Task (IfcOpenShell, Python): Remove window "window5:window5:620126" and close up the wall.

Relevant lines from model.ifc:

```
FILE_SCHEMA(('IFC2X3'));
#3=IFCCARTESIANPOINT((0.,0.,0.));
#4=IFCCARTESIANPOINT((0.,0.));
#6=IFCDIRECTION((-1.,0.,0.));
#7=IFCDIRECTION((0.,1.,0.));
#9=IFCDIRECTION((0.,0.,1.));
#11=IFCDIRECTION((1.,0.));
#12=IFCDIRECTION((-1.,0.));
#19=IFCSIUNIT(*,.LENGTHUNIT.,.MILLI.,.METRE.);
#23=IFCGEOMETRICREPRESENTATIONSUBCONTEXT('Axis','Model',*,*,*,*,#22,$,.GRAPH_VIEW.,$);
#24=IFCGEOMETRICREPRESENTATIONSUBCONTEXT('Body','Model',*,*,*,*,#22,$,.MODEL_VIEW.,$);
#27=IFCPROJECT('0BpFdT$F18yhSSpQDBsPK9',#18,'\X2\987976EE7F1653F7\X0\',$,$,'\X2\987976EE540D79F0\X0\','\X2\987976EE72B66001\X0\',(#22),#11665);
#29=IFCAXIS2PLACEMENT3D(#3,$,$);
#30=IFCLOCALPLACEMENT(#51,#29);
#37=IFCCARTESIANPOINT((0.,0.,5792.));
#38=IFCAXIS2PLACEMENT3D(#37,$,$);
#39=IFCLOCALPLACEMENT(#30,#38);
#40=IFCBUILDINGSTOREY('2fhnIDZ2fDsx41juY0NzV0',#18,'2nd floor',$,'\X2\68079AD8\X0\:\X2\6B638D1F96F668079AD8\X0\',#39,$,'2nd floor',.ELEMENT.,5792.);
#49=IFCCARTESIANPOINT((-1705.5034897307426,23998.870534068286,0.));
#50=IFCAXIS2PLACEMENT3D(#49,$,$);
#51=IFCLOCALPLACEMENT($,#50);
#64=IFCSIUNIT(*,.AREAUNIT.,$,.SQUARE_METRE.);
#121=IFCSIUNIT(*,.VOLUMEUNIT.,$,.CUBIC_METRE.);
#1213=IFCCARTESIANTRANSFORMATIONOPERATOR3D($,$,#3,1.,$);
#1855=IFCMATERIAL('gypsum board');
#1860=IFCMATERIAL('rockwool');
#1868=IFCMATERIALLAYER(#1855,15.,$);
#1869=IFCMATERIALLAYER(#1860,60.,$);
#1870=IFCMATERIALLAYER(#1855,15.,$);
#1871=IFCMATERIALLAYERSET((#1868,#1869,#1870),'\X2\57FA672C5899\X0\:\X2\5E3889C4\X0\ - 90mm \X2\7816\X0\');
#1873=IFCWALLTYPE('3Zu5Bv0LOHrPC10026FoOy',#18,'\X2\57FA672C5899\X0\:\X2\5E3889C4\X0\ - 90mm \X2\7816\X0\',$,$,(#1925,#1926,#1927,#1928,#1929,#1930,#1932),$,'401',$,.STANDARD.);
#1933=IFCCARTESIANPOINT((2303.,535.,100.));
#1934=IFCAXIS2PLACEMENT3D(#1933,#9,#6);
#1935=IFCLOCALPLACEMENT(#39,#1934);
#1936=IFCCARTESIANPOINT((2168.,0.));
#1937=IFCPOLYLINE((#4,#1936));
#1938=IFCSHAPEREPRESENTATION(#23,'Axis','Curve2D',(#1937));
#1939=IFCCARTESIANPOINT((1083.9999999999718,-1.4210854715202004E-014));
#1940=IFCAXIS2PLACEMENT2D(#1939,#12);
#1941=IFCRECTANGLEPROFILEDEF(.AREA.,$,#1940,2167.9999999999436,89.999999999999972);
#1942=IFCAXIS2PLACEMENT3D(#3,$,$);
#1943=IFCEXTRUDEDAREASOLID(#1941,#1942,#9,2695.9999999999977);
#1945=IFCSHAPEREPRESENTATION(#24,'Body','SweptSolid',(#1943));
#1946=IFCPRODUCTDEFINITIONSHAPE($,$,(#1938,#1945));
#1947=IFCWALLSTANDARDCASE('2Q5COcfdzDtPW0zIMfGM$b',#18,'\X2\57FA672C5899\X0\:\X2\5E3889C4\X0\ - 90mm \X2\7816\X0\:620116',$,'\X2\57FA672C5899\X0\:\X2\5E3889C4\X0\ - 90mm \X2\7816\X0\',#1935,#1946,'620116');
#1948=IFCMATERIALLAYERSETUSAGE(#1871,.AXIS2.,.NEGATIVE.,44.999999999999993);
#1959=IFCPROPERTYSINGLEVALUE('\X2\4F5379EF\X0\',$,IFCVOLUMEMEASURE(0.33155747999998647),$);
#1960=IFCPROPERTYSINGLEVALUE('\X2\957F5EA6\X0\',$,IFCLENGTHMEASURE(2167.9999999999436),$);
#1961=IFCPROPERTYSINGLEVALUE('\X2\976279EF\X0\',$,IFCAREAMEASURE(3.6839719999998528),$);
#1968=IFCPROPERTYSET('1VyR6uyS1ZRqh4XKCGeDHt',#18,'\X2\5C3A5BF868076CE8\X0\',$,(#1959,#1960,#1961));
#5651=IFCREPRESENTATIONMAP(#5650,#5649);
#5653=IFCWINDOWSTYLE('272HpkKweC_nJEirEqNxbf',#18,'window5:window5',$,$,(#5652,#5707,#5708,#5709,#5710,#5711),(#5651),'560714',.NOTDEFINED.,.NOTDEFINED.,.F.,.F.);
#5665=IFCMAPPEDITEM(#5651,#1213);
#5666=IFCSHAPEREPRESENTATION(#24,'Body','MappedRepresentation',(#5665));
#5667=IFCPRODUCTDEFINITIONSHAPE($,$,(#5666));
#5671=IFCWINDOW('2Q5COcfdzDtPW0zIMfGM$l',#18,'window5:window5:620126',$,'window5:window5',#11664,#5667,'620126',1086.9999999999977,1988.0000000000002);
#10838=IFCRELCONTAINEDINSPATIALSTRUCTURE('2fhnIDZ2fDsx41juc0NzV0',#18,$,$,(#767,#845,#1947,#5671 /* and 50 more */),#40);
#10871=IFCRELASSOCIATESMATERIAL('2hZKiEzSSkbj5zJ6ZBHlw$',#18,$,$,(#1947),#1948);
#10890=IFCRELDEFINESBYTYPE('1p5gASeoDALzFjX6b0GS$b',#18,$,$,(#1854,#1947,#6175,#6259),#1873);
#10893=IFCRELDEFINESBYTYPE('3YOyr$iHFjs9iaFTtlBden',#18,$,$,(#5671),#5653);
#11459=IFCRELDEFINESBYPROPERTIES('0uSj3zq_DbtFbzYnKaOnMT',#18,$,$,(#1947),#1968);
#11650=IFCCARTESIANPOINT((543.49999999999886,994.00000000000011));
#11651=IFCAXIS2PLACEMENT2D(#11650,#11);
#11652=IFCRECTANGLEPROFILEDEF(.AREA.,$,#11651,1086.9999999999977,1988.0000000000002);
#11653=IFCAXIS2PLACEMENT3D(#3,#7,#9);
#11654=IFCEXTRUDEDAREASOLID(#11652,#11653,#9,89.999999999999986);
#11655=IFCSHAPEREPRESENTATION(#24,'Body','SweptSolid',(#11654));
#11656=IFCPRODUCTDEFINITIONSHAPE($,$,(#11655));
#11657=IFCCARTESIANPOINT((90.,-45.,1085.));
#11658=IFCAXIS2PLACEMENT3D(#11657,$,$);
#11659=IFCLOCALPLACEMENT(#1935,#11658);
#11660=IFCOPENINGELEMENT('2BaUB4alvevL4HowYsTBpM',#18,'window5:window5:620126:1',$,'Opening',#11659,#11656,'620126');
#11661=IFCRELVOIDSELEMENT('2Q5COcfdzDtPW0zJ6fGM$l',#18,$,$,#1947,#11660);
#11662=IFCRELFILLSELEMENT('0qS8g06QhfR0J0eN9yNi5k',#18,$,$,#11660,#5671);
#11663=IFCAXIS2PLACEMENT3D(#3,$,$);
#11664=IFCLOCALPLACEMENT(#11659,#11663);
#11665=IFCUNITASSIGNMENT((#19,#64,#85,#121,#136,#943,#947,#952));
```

```python
import ifcopenshell
import ifcopenshell.api.feature
import ifcopenshell.api.pset
import ifcopenshell.api.root
import ifcopenshell.geom
import ifcopenshell.util.element
import ifcopenshell.util.shape
import ifcopenshell.util.unit

model = ifcopenshell.open("model.ifc")
area_scale = ifcopenshell.util.unit.calculate_unit_scale(model, "AREAUNIT")
volume_scale = ifcopenshell.util.unit.calculate_unit_scale(model, "VOLUMEUNIT")
settings = ifcopenshell.geom.settings()


def volume(element):
    """Net volume in cubic metres, openings subtracted."""
    shape = ifcopenshell.geom.create_shape(settings, element)
    return ifcopenshell.util.shape.get_volume(shape.geometry)


window = model.by_guid("2Q5COcfdzDtPW0zIMfGM$l")
opening = window.FillsVoids[0].RelatingOpeningElement
wall = opening.VoidsElements[0].RelatingBuildingElement
before = volume(wall)

ifcopenshell.api.root.remove_product(model, product=window)
ifcopenshell.api.feature.remove_feature(model, feature=opening)

after = volume(wall)
thickness = 0.09  # wall thickness in metres

# Update the wall's stored quantities.
pset = model.by_id(ifcopenshell.util.element.get_pset(wall, "尺寸标注", should_inherit=False)["id"])
ifcopenshell.api.pset.edit_pset(model, pset=pset, properties={
    "体积": model.create_entity("IfcVolumeMeasure", after / volume_scale),
    "面积": model.create_entity("IfcAreaMeasure", after / thickness / area_scale),
})

print(f"wall volume {before:.3f} -> {after:.3f} m3")

model.write("model_rev.ifc")
```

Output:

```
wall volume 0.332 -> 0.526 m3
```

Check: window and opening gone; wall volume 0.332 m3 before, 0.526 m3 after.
